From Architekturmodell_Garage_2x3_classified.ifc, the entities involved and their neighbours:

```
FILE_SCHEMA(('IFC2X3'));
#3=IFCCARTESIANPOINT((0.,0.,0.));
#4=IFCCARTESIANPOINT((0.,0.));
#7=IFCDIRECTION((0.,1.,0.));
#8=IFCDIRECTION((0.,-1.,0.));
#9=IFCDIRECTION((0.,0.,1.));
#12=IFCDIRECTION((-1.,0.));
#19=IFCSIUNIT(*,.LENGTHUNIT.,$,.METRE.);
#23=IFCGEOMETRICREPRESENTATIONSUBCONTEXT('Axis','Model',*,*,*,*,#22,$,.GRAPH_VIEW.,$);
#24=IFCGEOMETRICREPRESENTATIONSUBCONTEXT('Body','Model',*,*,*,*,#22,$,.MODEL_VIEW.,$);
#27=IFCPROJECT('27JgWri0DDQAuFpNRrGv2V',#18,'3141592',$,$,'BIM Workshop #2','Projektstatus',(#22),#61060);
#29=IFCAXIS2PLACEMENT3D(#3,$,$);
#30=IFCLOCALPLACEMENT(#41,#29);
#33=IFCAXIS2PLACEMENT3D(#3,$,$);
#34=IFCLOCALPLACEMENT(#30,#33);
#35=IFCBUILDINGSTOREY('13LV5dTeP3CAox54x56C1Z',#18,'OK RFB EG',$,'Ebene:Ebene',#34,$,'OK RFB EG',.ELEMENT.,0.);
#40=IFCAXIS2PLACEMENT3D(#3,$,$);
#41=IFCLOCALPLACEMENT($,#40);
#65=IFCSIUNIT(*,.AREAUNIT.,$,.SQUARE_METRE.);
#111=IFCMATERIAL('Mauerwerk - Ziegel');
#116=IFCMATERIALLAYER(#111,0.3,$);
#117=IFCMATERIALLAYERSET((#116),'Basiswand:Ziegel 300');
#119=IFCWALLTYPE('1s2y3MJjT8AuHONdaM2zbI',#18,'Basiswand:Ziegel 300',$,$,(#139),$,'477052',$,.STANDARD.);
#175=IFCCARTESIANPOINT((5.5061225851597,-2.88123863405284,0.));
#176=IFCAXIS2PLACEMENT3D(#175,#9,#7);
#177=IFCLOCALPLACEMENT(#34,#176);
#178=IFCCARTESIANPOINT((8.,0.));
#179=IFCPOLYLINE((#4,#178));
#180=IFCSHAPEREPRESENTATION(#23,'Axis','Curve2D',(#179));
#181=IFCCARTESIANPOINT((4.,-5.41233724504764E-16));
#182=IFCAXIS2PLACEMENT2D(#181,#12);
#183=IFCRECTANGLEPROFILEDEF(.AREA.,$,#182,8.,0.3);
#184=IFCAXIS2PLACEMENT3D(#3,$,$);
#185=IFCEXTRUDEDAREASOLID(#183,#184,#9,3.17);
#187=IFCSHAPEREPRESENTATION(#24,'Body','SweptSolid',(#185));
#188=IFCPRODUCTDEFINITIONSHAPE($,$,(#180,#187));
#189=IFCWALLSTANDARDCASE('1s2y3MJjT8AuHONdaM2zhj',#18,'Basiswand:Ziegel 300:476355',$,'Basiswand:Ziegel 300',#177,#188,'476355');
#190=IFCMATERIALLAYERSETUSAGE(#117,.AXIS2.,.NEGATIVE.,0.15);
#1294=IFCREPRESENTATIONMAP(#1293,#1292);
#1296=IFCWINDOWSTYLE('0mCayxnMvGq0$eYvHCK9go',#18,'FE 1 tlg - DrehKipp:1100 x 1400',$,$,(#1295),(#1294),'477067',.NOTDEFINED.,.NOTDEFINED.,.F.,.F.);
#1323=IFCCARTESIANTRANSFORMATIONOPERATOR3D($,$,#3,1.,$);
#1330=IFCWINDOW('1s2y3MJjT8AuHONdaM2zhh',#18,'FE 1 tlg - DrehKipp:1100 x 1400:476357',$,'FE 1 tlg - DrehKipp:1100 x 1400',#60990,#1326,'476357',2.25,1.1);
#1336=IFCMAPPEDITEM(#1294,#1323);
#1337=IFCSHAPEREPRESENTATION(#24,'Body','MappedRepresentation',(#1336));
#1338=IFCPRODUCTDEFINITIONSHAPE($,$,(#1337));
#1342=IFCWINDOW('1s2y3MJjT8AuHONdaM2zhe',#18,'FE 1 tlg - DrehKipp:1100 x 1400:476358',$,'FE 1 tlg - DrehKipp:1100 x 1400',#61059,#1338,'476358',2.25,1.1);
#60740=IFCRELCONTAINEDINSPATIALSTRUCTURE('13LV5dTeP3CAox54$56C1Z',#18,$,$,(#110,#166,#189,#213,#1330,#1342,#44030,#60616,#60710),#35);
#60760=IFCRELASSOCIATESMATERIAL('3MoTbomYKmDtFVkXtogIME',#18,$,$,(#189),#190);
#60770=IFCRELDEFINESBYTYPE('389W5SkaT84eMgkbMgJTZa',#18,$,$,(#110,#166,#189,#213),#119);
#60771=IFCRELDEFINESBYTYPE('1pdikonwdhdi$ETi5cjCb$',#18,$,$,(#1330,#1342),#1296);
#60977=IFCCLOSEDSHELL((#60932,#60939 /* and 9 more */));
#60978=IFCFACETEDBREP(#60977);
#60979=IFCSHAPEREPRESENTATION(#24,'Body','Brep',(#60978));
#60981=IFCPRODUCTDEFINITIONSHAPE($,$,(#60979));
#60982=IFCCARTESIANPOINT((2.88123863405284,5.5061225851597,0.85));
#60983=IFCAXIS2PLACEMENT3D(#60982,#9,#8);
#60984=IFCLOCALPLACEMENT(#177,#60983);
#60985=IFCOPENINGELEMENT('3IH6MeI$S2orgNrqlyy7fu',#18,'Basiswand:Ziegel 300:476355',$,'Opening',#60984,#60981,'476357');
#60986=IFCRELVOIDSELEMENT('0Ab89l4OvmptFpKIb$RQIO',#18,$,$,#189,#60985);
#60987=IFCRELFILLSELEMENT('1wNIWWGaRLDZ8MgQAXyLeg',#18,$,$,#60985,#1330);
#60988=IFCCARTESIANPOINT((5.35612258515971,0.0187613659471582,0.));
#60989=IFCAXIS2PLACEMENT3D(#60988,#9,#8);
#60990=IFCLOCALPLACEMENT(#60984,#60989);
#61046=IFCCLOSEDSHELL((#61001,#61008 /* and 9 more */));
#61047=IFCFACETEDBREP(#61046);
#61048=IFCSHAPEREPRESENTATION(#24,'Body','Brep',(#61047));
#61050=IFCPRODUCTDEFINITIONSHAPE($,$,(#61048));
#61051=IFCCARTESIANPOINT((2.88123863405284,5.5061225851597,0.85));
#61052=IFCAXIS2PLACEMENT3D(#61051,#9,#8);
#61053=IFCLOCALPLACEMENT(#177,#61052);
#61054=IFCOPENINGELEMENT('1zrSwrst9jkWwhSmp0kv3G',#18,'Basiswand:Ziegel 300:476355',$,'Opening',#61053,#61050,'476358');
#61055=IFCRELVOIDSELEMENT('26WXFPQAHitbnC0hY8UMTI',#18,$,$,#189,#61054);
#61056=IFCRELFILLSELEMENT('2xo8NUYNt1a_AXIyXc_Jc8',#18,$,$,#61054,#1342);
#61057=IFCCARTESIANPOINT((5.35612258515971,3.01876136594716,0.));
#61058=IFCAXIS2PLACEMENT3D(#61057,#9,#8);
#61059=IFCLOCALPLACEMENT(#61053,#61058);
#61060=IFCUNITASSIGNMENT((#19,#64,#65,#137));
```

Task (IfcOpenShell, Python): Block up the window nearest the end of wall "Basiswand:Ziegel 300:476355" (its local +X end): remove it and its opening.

```python
import ifcopenshell
import ifcopenshell.api.feature
import ifcopenshell.api.root
import ifcopenshell.geom
import ifcopenshell.util.shape

model = ifcopenshell.open("Architekturmodell_Garage_2x3_classified.ifc")
settings = ifcopenshell.geom.settings()


def volume(element):
    """Net volume in cubic metres, openings subtracted."""
    shape = ifcopenshell.geom.create_shape(settings, element)
    return ifcopenshell.util.shape.get_volume(shape.geometry)


window = model.by_guid("1s2y3MJjT8AuHONdaM2zhe")
opening = window.FillsVoids[0].RelatingOpeningElement
wall = opening.VoidsElements[0].RelatingBuildingElement
before = volume(wall)

ifcopenshell.api.root.remove_product(model, product=window)
ifcopenshell.api.feature.remove_feature(model, feature=opening)

after = volume(wall)

print(f"wall volume {before:.3f} -> {after:.3f} m3")

model.write("Architekturmodell_Garage_2x3_classified_rev.ifc")
```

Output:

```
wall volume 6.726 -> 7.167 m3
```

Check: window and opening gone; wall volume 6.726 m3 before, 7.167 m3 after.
